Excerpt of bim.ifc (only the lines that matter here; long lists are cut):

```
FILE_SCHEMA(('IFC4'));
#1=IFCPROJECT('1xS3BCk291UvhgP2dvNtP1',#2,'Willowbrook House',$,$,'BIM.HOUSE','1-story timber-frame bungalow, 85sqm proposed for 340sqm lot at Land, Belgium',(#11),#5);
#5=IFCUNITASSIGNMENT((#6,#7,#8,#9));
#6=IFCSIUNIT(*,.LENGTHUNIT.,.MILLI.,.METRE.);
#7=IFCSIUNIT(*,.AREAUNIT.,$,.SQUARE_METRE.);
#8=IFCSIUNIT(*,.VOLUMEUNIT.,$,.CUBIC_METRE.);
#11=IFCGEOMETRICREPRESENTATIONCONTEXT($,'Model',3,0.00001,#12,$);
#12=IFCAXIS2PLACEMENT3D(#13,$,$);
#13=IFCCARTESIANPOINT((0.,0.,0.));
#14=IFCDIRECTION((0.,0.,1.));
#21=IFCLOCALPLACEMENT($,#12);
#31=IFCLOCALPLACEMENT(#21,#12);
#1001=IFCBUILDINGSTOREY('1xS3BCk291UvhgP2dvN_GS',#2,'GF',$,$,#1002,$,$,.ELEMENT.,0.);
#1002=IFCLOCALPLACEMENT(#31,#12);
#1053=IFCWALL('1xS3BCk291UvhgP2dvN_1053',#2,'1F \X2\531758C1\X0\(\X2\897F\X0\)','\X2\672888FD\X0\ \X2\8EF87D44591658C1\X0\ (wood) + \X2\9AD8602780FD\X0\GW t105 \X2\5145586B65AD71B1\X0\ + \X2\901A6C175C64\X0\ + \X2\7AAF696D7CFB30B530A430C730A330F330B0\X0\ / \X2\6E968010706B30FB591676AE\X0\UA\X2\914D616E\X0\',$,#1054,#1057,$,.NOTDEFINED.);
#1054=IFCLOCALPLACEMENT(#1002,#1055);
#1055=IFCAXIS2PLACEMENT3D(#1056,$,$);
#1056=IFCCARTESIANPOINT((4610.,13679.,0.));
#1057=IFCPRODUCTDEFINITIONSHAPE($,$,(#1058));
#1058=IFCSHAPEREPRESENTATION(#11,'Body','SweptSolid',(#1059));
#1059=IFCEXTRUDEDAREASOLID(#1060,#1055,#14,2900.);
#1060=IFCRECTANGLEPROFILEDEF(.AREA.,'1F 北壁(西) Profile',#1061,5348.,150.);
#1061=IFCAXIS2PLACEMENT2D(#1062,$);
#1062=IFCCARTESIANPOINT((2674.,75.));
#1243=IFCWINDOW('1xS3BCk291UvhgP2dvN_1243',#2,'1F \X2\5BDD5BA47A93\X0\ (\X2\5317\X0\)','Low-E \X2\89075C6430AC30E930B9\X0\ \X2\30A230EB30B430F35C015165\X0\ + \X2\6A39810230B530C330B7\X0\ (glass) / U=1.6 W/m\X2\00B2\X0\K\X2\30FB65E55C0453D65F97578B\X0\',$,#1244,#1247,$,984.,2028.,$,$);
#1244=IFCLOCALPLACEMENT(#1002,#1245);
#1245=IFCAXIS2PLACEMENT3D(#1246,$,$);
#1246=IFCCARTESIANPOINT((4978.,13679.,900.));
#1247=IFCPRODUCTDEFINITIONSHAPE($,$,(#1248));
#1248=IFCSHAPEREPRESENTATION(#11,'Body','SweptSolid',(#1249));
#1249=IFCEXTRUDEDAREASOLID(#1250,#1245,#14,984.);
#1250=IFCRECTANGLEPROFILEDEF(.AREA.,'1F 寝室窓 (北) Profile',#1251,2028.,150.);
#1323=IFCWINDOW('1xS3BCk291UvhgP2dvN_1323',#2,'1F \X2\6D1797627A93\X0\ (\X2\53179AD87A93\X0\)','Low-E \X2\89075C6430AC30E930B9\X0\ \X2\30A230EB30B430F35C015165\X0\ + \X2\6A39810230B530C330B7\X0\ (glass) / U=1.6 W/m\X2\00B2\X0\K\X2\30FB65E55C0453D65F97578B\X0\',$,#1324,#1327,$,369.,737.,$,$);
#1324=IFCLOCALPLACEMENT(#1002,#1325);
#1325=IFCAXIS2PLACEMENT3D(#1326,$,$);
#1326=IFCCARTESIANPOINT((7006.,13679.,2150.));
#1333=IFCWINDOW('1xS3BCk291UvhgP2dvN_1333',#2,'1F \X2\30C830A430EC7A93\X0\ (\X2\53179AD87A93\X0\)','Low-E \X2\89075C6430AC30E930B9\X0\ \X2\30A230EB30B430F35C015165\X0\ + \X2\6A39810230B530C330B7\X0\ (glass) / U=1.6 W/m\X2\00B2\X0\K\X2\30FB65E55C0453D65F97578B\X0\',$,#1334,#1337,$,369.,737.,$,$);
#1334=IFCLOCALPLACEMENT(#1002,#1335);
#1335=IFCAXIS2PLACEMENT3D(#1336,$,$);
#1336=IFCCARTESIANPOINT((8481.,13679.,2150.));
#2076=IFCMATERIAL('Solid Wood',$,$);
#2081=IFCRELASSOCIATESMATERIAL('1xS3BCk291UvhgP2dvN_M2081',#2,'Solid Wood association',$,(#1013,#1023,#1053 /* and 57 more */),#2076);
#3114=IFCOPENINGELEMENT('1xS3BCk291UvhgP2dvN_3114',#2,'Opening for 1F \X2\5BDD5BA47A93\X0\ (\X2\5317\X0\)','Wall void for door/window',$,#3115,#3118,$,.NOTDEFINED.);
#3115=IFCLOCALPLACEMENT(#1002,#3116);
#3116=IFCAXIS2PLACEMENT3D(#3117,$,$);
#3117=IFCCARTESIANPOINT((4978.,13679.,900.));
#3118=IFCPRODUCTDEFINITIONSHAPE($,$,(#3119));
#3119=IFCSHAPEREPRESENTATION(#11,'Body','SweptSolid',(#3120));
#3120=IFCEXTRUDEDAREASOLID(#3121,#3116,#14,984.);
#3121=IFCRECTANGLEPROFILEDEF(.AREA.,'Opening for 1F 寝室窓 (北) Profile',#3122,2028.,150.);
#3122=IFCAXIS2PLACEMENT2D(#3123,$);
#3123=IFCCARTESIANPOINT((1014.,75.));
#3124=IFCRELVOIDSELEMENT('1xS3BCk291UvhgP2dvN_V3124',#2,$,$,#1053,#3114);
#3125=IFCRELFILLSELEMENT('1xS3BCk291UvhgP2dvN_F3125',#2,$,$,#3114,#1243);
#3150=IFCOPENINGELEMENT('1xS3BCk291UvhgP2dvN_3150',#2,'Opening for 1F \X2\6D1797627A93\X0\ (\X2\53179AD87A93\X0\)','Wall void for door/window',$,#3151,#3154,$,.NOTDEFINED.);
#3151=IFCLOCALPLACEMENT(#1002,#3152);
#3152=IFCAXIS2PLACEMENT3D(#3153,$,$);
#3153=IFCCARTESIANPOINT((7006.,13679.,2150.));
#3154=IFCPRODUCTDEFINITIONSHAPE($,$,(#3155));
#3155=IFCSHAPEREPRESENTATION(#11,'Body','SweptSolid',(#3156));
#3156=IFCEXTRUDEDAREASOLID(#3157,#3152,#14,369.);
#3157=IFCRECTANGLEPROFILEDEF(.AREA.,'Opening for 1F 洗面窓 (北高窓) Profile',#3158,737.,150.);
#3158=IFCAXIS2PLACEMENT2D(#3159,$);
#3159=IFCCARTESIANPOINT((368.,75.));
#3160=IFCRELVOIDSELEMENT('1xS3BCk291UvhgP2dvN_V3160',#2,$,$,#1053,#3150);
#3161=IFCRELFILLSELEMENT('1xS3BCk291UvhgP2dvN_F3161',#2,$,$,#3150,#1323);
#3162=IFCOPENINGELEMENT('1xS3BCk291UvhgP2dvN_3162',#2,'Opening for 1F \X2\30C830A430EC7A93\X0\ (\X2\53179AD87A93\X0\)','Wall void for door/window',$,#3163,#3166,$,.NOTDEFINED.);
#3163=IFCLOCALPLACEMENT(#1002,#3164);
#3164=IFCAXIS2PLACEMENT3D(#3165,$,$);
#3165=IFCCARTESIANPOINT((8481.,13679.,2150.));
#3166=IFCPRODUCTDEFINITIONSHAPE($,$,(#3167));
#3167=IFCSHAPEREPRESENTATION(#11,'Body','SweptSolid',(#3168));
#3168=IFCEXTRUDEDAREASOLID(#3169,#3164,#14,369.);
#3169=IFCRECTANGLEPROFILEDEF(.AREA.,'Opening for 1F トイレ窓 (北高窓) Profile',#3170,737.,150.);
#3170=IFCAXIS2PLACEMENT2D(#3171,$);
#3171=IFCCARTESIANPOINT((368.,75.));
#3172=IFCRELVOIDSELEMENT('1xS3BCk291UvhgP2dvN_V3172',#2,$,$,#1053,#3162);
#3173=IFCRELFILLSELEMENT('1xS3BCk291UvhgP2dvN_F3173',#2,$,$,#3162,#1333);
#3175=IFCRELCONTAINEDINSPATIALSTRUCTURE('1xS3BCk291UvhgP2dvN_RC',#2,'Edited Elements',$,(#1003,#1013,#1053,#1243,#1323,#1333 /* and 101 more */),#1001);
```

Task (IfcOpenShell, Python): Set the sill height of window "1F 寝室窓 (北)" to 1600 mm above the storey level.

```python
import numpy as np
import ifcopenshell
import ifcopenshell.api.geometry
import ifcopenshell.geom
import ifcopenshell.util.element
import ifcopenshell.util.placement
import ifcopenshell.util.shape
import ifcopenshell.util.unit

model = ifcopenshell.open("bim.ifc")
unit_scale = ifcopenshell.util.unit.calculate_unit_scale(model)

window = model.by_guid("1xS3BCk291UvhgP2dvN_1243")
opening = window.FillsVoids[0].RelatingOpeningElement
storey = ifcopenshell.util.element.get_container(window, ifc_class="IfcBuildingStorey")
level = ifcopenshell.util.placement.get_local_placement(storey.ObjectPlacement)[2, 3]

# The opening's origin need not be at the sill, so measure its lowest point.
shape = ifcopenshell.geom.create_shape(ifcopenshell.geom.settings(), opening)
bottom = ifcopenshell.util.shape.get_shape_bottom_elevation(shape, shape.geometry) / unit_scale
dz = level + 1600.0 - bottom

shift = np.array([0.0, 0.0, dz])
# The window is not placed relative to its opening, so move both.
for product in (opening, window):
    matrix = ifcopenshell.util.placement.get_local_placement(product.ObjectPlacement)
    matrix[:3, 3] += shift
    ifcopenshell.api.geometry.edit_object_placement(model, product=product, matrix=matrix, is_si=False)

print(f"moved by {dz * unit_scale:+.3f} m")

model.write("bim-out.ifc")
```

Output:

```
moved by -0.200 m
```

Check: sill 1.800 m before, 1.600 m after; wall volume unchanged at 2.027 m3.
